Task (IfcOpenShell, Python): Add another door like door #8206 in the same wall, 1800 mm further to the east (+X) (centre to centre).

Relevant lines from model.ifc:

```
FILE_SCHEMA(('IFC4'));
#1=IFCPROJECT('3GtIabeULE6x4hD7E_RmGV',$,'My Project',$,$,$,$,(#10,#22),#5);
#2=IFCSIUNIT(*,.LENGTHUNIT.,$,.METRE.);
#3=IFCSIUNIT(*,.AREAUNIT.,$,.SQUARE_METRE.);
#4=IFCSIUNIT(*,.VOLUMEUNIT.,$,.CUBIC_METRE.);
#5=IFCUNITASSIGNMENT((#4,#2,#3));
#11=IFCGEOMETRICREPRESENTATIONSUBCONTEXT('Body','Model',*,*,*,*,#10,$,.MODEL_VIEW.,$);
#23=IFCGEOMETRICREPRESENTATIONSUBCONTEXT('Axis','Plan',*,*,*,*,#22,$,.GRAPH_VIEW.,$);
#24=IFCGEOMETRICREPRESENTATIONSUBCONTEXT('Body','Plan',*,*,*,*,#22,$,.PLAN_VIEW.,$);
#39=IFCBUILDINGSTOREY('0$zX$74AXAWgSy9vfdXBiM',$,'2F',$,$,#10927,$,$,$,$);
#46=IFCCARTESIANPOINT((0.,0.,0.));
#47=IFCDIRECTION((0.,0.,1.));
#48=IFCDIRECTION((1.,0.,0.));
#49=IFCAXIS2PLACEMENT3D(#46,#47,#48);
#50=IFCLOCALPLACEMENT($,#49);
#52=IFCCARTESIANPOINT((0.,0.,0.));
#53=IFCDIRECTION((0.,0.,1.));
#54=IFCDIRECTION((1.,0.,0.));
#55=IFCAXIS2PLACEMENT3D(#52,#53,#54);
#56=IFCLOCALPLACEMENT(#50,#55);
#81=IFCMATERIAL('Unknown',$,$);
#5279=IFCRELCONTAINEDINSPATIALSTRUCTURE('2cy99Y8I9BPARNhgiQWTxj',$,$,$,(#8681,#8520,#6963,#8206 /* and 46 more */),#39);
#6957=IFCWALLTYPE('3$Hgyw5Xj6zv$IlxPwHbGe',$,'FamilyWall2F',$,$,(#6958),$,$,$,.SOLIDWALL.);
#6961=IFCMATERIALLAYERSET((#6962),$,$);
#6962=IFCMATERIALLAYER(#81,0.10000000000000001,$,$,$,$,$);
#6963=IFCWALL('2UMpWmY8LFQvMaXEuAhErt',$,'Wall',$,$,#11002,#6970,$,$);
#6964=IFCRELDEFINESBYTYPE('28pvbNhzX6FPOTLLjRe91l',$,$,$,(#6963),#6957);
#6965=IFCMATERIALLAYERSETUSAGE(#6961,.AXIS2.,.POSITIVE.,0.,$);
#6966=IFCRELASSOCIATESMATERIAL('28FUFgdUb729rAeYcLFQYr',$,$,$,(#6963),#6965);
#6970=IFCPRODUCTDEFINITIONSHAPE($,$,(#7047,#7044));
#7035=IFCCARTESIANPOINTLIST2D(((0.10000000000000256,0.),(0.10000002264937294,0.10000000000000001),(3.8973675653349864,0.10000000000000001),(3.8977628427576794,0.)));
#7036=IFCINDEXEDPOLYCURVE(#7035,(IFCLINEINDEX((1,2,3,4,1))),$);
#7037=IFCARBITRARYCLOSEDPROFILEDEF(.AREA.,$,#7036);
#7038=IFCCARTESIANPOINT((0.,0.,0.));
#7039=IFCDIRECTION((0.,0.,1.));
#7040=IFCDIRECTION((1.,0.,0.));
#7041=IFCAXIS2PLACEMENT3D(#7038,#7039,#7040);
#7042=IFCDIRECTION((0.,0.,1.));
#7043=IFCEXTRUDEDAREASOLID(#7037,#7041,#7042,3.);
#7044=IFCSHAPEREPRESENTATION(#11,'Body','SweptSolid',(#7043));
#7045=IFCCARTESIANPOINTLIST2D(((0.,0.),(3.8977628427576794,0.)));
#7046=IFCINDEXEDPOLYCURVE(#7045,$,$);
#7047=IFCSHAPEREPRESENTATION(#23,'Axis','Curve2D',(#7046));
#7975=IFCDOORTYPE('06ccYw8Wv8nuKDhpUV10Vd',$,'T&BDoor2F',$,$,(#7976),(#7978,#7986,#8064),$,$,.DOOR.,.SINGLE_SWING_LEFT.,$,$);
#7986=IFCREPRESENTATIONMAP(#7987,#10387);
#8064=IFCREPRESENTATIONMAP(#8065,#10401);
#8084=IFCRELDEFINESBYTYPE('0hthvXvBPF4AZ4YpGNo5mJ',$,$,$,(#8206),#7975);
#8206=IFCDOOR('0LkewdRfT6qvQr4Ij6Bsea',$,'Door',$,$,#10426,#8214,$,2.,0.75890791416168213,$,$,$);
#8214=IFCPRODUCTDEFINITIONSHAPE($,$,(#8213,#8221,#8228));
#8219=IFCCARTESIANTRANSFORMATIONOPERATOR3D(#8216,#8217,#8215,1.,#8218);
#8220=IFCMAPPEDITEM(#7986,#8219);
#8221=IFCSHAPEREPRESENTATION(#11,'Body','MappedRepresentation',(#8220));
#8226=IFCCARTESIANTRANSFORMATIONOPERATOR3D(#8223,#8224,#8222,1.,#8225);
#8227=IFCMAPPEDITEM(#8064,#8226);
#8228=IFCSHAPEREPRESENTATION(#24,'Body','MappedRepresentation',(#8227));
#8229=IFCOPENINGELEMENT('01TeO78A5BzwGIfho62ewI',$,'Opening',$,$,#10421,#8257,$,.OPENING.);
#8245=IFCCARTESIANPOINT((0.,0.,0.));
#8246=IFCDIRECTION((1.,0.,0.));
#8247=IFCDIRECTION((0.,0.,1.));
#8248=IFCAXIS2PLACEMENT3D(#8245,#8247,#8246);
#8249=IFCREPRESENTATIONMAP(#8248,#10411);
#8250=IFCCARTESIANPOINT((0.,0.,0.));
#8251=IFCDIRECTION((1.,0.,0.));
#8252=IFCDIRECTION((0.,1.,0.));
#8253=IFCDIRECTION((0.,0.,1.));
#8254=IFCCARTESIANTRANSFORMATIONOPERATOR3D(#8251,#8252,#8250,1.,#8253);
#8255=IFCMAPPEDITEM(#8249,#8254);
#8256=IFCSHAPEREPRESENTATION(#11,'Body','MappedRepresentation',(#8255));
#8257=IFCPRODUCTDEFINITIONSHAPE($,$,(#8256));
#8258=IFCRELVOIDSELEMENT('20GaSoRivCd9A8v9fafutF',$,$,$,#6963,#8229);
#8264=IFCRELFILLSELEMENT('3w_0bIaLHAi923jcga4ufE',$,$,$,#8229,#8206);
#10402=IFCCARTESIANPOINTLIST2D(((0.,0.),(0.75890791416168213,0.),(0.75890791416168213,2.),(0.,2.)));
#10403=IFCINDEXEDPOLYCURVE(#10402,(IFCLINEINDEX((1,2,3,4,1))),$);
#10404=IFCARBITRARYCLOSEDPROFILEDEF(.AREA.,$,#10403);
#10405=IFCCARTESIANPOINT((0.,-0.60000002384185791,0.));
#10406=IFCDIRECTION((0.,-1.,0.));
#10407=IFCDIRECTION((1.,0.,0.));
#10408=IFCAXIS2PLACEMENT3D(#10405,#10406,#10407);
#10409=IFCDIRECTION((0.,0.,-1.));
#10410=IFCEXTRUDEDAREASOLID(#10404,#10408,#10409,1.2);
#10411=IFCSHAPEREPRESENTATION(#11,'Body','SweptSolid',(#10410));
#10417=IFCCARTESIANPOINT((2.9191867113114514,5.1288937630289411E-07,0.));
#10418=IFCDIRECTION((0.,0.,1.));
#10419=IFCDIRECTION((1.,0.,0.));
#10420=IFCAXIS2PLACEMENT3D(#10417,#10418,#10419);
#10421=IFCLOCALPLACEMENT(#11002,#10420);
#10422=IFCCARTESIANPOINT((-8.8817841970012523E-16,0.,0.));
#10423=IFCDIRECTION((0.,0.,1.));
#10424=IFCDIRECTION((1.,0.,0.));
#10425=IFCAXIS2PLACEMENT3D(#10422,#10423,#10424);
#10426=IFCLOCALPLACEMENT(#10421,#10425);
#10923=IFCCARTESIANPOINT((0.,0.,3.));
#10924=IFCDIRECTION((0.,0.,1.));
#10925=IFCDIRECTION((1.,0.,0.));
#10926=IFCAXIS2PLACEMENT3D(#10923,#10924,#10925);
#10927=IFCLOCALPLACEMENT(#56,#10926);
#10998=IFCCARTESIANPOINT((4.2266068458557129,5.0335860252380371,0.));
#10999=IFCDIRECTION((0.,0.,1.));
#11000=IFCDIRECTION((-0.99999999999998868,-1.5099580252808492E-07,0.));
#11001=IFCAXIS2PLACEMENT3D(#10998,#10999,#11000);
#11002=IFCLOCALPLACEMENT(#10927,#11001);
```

```python
import ifcopenshell
import ifcopenshell.api.feature
import ifcopenshell.api.geometry
import ifcopenshell.api.root
import ifcopenshell.geom
import ifcopenshell.util.element
import ifcopenshell.util.placement
import ifcopenshell.util.shape
import ifcopenshell.util.unit

model = ifcopenshell.open("model.ifc")
unit_scale = ifcopenshell.util.unit.calculate_unit_scale(model)
settings = ifcopenshell.geom.settings()


def volume(element):
    """Net volume in cubic metres, openings subtracted."""
    shape = ifcopenshell.geom.create_shape(settings, element)
    return ifcopenshell.util.shape.get_volume(shape.geometry)


door = model.by_guid("0LkewdRfT6qvQr4Ij6Bsea")
opening = door.FillsVoids[0].RelatingOpeningElement
wall = opening.VoidsElements[0].RelatingBuildingElement
before = volume(wall)
shift = ifcopenshell.util.placement.get_local_placement(wall.ObjectPlacement)[:3, 0] * -1.8 / unit_scale

# copy_class copies the void relationship, type, container and properties, but no geometry.
new_opening = ifcopenshell.api.root.copy_class(model, product=opening)
new_opening.Representation = ifcopenshell.util.element.copy_deep(
    model, opening.Representation, exclude=["IfcGeometricRepresentationContext", "IfcRepresentationMap"]
)
new_door = ifcopenshell.api.root.copy_class(model, product=door)
new_door.Representation = ifcopenshell.util.element.copy_deep(
    model, door.Representation, exclude=["IfcGeometricRepresentationContext", "IfcRepresentationMap"]
)
ifcopenshell.api.feature.add_filling(model, opening=new_opening, element=new_door)

for old, new in ((opening, new_opening), (door, new_door)):
    matrix = ifcopenshell.util.placement.get_local_placement(old.ObjectPlacement)
    matrix[:3, 3] += shift
    ifcopenshell.api.geometry.edit_object_placement(model, product=new, matrix=matrix, is_si=False)

after = volume(wall)

print(f"wall volume {before:.3f} -> {after:.3f} m3")

model.write("model-out.ifc")
```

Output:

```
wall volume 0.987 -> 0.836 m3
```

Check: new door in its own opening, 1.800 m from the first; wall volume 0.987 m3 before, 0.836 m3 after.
